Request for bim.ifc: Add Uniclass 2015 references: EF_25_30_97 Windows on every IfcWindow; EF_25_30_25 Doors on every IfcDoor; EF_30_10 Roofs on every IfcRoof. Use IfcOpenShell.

First a look at what the model holds.

```python
import ifcopenshell

model = ifcopenshell.open("bim.ifc")
print(model.schema)
print("classifications:", [c.Name for c in model.by_type("IfcClassification")])
for ifc_class in ("IfcDoor", "IfcRoof", "IfcStair", "IfcWall", "IfcWindow"):
    print(ifc_class, len(model.by_type(ifc_class)))
```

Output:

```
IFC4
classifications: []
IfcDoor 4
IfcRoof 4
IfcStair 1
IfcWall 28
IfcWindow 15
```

```python
import ifcopenshell
import ifcopenshell.api.classification

model = ifcopenshell.open("bim.ifc")

system = ifcopenshell.api.classification.add_classification(model, classification="Uniclass 2015")

codes = {
    "IfcWindow": ("EF_25_30_97", "Windows"),
    "IfcDoor": ("EF_25_30_25", "Doors"),
    "IfcRoof": ("EF_30_10", "Roofs"),
}
for ifc_class, (code, name) in codes.items():
    products = model.by_type(ifc_class)
    ifcopenshell.api.classification.add_reference(
        model, products=products, classification=system, identification=code, name=name
    )
    print(code, len(products))

model.write("bim_rev.ifc")
```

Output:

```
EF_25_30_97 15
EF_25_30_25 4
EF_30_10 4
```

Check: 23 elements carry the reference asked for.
